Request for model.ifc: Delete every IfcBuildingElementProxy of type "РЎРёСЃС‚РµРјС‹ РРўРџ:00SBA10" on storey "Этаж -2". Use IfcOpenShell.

First a look at what the model holds.

```python
import ifcopenshell
import ifcopenshell.util.element

model = ifcopenshell.open("model.ifc")
print(model.schema)
storey = next(s for s in model.by_type("IfcBuildingStorey") if s.Name == "Этаж -2")
proxies = [e for e in ifcopenshell.util.element.get_decomposition(storey) if e.is_a("IfcBuildingElementProxy")]
seen = {}
for e in proxies:
    element_type = ifcopenshell.util.element.get_type(e)
    name = element_type.Name if element_type not in (None, e) else None
    seen[name] = seen.get(name, 0) + 1
for name, count in sorted(seen.items(), key=str):
    print(count, "x", name)
```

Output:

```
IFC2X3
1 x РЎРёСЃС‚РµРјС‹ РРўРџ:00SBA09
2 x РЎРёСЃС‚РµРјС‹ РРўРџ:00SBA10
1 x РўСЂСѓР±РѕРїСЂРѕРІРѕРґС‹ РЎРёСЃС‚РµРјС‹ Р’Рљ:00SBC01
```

```python
import ifcopenshell
import ifcopenshell.api.root
import ifcopenshell.util.element

model = ifcopenshell.open("model.ifc")

storey = next(s for s in model.by_type("IfcBuildingStorey") if s.Name == "Этаж -2")
proxies = [e for e in ifcopenshell.util.element.get_decomposition(storey) if e.is_a("IfcBuildingElementProxy")]
targets = [e for e in proxies if (t := ifcopenshell.util.element.get_type(e)) not in (None, e) and t.Name == 'РЎРёСЃС‚РµРјС‹ Р\x98РўРџ:00SBA10']

for e in targets:
    ifcopenshell.api.root.remove_product(model, product=e)
print(len(targets), "removed")

model.write("model_updated.ifc")
```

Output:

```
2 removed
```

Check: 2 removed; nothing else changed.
